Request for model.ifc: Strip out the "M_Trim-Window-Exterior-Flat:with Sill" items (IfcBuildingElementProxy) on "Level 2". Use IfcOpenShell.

First a look at what the model holds.

```python
import ifcopenshell
import ifcopenshell.util.element

model = ifcopenshell.open("model.ifc")
print(model.schema)
storey = next(s for s in model.by_type("IfcBuildingStorey") if s.Name == "Level 2")
proxies = [e for e in ifcopenshell.util.element.get_decomposition(storey) if e.is_a("IfcBuildingElementProxy")]
seen = {}
for e in proxies:
    element_type = ifcopenshell.util.element.get_type(e)
    name = element_type.Name if element_type not in (None, e) else None
    seen[name] = seen.get(name, 0) + 1
for name, count in sorted(seen.items(), key=str):
    print(count, "x", name)
```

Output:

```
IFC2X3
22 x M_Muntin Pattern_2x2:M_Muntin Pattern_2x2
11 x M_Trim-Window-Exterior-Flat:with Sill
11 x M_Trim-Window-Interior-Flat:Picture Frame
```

```python
import ifcopenshell
import ifcopenshell.api.root
import ifcopenshell.util.element

model = ifcopenshell.open("model.ifc")

storey = next(s for s in model.by_type("IfcBuildingStorey") if s.Name == "Level 2")
proxies = [e for e in ifcopenshell.util.element.get_decomposition(storey) if e.is_a("IfcBuildingElementProxy")]
targets = [e for e in proxies if (t := ifcopenshell.util.element.get_type(e)) not in (None, e) and t.Name == "M_Trim-Window-Exterior-Flat:with Sill"]

for e in targets:
    ifcopenshell.api.root.remove_product(model, product=e)
print(len(targets), "removed")

model.write("model_rev.ifc")
```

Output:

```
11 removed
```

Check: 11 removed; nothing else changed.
